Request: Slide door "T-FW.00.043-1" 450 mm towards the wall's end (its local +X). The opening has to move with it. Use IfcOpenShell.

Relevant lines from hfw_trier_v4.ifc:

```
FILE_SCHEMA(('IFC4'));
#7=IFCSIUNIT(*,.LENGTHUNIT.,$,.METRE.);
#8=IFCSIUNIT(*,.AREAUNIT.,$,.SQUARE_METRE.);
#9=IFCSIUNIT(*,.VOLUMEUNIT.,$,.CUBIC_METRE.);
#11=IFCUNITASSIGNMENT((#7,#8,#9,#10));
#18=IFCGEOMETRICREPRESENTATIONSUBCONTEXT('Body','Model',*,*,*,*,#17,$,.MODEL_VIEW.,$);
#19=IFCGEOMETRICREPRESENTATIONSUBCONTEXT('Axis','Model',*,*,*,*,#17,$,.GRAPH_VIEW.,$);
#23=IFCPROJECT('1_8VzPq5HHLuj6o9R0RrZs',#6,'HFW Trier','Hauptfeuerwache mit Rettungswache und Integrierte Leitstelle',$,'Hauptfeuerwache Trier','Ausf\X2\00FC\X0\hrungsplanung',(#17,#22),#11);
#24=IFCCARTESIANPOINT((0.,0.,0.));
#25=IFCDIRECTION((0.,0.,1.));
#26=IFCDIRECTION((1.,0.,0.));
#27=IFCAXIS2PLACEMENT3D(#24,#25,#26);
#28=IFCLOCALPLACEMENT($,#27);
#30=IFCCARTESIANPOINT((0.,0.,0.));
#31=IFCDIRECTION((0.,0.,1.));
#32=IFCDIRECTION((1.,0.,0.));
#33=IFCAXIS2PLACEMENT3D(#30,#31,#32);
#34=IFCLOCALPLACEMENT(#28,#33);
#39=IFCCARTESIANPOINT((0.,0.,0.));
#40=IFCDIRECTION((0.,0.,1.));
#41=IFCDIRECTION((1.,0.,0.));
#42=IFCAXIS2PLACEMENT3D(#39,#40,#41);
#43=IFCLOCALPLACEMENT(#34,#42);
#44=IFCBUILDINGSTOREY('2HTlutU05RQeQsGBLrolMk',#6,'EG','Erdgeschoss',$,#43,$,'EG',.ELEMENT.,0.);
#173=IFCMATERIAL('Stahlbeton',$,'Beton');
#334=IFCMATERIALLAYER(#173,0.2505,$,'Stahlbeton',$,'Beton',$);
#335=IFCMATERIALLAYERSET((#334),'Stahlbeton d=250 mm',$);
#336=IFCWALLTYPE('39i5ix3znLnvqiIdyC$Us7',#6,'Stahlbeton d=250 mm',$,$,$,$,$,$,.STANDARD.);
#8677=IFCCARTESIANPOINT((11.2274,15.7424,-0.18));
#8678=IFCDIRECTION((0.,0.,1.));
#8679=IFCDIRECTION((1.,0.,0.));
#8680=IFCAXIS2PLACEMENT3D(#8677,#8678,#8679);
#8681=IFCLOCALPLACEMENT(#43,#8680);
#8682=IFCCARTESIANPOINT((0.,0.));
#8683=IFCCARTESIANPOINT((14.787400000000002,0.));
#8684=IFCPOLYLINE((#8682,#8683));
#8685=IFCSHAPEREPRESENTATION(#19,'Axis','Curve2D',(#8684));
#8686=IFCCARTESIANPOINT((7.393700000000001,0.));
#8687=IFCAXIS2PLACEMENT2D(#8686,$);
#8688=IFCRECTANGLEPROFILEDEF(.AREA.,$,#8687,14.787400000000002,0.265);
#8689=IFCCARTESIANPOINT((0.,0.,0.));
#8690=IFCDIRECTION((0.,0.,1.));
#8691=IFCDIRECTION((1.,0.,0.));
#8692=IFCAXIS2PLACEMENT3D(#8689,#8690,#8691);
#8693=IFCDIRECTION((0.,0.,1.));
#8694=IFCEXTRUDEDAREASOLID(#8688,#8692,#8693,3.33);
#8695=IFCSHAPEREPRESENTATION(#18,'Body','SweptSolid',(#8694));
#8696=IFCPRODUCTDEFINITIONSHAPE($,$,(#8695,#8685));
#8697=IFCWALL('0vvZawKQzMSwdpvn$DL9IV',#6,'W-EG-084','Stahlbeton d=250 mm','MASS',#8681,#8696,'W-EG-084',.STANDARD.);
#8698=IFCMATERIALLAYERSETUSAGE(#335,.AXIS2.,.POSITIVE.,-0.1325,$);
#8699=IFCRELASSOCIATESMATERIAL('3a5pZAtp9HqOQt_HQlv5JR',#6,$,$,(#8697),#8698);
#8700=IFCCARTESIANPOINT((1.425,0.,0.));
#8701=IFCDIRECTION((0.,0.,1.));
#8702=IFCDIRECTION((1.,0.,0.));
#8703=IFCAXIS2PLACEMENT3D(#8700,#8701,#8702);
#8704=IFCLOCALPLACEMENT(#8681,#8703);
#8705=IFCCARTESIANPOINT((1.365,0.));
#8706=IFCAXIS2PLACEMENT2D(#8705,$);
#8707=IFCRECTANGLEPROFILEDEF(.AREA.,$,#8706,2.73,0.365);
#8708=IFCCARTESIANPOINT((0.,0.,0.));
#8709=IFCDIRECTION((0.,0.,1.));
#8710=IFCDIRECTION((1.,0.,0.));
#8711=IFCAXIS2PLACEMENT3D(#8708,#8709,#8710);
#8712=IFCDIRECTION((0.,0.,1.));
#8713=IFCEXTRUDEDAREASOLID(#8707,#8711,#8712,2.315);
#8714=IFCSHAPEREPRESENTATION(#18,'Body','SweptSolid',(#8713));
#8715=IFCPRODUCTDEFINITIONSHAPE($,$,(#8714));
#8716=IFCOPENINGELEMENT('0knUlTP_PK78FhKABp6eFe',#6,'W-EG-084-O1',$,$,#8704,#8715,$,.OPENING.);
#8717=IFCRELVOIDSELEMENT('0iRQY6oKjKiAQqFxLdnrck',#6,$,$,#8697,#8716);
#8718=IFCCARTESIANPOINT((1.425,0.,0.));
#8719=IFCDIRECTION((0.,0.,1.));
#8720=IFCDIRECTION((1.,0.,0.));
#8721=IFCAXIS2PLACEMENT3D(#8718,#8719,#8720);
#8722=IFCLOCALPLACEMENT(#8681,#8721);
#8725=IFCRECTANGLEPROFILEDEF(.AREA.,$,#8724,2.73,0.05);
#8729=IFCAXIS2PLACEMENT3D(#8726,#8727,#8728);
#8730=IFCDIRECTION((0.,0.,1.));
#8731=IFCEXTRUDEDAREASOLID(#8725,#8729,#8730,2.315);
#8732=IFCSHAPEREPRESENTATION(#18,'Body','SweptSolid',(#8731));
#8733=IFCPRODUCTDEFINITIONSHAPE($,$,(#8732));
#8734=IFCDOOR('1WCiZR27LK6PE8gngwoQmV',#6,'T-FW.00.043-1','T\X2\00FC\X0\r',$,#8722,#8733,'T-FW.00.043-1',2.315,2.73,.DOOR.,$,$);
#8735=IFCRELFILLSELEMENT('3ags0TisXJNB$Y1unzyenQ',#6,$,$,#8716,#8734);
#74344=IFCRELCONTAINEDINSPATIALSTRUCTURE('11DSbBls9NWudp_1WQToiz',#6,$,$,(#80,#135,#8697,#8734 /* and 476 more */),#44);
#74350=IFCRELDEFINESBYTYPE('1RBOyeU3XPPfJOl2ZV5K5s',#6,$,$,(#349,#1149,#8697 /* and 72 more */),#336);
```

```python
import ifcopenshell
import ifcopenshell.api.geometry
import ifcopenshell.util.placement

model = ifcopenshell.open("hfw_trier_v4.ifc")

door = model.by_id(8734)
opening = door.FillsVoids[0].RelatingOpeningElement
wall = opening.VoidsElements[0].RelatingBuildingElement

wall_matrix = ifcopenshell.util.placement.get_local_placement(wall.ObjectPlacement)
shift = wall_matrix[:3, 0] * 0.45
before = ifcopenshell.util.placement.get_local_placement(door.ObjectPlacement)[:3, 3].copy()

# The door is not placed relative to its opening, so move both.
for product in (opening, door):
    matrix = ifcopenshell.util.placement.get_local_placement(product.ObjectPlacement)
    matrix[:3, 3] += shift
    ifcopenshell.api.geometry.edit_object_placement(model, product=product, matrix=matrix, is_si=False)

after = ifcopenshell.util.placement.get_local_placement(door.ObjectPlacement)[:3, 3]
print("door moved by", (after - before).round(3) + 0.0)

model.write("hfw_trier_v4_edited.ifc")
```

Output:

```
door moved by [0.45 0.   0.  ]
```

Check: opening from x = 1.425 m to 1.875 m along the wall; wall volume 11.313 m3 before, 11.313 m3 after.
